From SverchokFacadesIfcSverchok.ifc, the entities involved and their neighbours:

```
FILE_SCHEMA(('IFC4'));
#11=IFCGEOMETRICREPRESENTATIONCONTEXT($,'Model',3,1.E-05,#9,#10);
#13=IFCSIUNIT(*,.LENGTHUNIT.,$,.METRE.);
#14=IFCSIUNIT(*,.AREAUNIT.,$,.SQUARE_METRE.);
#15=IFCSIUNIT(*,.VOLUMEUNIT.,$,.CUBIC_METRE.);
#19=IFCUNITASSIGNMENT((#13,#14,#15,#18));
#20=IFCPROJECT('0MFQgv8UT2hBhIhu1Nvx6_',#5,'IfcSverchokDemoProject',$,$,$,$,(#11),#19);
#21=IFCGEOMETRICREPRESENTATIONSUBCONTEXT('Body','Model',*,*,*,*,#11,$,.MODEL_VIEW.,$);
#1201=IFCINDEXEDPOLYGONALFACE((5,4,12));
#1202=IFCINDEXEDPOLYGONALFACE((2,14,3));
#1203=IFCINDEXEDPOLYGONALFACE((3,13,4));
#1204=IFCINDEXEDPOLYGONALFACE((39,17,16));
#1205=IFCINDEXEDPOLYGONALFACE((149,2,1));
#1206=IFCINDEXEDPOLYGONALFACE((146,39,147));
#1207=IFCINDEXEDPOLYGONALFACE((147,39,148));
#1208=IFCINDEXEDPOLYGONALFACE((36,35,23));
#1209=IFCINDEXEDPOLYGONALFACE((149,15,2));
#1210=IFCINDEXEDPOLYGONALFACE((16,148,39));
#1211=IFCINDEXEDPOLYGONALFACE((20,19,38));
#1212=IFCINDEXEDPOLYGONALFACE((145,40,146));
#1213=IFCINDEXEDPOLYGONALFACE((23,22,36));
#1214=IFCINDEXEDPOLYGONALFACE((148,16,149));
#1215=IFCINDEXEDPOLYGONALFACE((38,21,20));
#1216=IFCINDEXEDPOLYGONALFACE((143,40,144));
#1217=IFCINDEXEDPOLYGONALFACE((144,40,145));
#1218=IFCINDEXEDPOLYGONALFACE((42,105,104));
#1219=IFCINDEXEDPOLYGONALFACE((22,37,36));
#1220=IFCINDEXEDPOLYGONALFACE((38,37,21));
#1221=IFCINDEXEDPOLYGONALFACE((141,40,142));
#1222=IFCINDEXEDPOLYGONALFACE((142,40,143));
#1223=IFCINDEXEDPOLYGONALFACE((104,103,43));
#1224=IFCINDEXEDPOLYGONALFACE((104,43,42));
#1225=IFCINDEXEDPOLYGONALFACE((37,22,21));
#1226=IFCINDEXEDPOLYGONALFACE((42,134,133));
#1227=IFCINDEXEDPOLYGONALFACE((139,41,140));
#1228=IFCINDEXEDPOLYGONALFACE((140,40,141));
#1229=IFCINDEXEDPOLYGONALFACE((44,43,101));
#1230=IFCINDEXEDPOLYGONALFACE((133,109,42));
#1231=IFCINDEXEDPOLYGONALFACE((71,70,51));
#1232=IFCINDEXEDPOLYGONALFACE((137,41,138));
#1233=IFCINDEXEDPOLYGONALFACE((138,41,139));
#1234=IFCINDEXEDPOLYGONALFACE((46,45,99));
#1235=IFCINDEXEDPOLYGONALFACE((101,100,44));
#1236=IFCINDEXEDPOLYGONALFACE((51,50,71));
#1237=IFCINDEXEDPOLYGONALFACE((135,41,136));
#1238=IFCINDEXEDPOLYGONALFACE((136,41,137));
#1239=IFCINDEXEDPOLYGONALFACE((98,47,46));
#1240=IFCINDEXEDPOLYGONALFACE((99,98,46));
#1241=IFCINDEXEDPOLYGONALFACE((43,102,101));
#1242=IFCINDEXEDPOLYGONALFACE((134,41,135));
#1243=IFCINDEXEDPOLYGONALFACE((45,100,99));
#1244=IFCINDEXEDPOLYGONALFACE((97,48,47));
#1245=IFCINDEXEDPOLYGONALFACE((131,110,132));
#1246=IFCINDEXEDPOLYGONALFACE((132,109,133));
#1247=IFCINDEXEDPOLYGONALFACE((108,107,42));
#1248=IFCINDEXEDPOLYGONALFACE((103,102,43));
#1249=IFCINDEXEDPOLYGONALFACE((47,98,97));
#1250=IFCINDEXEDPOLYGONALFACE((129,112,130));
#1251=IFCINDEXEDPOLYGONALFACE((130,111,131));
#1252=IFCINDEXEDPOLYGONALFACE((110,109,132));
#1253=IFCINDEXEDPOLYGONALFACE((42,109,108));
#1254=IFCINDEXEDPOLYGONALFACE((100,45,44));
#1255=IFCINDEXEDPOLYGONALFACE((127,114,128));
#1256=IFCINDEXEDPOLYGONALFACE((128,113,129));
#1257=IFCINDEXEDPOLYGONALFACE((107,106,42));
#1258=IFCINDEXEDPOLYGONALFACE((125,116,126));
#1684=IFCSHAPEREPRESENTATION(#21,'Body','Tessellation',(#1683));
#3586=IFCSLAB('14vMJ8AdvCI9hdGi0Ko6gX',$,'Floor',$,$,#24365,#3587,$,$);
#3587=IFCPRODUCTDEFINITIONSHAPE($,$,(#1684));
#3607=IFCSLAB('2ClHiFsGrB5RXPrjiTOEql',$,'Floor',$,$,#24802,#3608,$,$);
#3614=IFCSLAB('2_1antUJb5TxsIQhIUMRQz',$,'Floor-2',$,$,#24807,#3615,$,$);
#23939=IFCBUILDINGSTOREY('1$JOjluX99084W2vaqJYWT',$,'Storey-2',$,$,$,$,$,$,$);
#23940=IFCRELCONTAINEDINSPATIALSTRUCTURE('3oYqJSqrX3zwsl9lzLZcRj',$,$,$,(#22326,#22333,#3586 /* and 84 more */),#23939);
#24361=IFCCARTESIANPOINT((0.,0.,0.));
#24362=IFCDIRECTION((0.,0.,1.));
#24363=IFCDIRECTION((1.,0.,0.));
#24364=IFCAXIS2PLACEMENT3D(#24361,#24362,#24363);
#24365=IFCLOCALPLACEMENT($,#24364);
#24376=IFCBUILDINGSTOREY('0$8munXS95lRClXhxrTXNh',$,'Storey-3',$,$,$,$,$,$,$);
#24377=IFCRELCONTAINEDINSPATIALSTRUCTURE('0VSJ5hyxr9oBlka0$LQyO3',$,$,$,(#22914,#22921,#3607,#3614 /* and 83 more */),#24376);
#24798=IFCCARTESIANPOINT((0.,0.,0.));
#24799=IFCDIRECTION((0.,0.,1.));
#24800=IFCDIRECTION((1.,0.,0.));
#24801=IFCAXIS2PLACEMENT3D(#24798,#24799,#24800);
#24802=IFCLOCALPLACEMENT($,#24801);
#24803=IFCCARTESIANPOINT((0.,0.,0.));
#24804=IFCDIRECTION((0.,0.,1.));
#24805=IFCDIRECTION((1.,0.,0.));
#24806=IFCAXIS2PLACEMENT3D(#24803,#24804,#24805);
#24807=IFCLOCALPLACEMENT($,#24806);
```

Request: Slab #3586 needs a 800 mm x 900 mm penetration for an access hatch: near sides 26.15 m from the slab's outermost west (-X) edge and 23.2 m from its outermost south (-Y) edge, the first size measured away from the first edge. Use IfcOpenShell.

```python
import numpy as np
import ifcopenshell
import ifcopenshell.api.feature
import ifcopenshell.api.geometry
import ifcopenshell.api.root
import ifcopenshell.geom
import ifcopenshell.util.placement
import ifcopenshell.util.representation
import ifcopenshell.util.shape
import ifcopenshell.util.unit

model = ifcopenshell.open("SverchokFacadesIfcSverchok.ifc")
unit_scale = ifcopenshell.util.unit.calculate_unit_scale(model)
settings = ifcopenshell.geom.settings()


def volume(element):
    """Net volume in cubic metres, openings subtracted."""
    shape = ifcopenshell.geom.create_shape(settings, element)
    return ifcopenshell.util.shape.get_volume(shape.geometry)


slab = model.by_guid("14vMJ8AdvCI9hdGi0Ko6gX")
before = volume(slab)

# Extent in the slab's own axes, in metres. The edges named are its -X and -Y sides.
slab_shape = ifcopenshell.geom.create_shape(settings, slab)
vertices = ifcopenshell.util.shape.get_vertices(slab_shape.geometry)
x_min, y_min, bottom = vertices.min(axis=0)
top = vertices[:, 2].max()

opening = ifcopenshell.api.root.create_entity(model, ifc_class="IfcOpeningElement", name="Access hatch opening", predefined_type="OPENING")
context = ifcopenshell.util.representation.get_context(model, "Model", "Body", "MODEL_VIEW")
width, depth = 0.8, 0.9
outline = [(0.0, 0.0), (width, 0.0), (width, depth), (0.0, depth), (0.0, 0.0)]
# Overshoot both faces by 50 mm so the cut is clean.
shape = ifcopenshell.api.geometry.add_slab_representation(
    model, context=context, depth=top - bottom + 0.1, polyline=outline
)
ifcopenshell.api.geometry.assign_representation(model, product=opening, representation=shape)

matrix = ifcopenshell.util.placement.get_local_placement(slab.ObjectPlacement)
matrix[:, 3] = matrix @ np.append(np.array([x_min + 26.15, y_min + 23.2, bottom - 0.05]) / unit_scale, 1.0)
ifcopenshell.api.geometry.edit_object_placement(model, product=opening, matrix=matrix, is_si=False)
ifcopenshell.api.feature.add_feature(model, feature=opening, element=slab)

after = volume(slab)

print(f"slab volume {before:.3f} -> {after:.3f} m3")

model.write("SverchokFacadesIfcSverchok_rev.ifc")
```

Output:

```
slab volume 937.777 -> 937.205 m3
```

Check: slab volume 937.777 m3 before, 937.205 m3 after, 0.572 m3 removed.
